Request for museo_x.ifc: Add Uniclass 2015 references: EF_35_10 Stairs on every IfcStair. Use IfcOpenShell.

First a look at what the model holds.

```python
import ifcopenshell

model = ifcopenshell.open("museo_x.ifc")
print(model.schema)
print("classifications:", [c.Name for c in model.by_type("IfcClassification")])
for ifc_class in ("IfcDoor", "IfcRoof", "IfcStair", "IfcWall", "IfcWindow"):
    print(ifc_class, len(model.by_type(ifc_class)))
```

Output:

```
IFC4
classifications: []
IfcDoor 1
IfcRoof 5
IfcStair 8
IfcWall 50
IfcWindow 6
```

```python
import ifcopenshell
import ifcopenshell.api.classification

model = ifcopenshell.open("museo_x.ifc")

system = ifcopenshell.api.classification.add_classification(model, classification="Uniclass 2015")

codes = {
    "IfcStair": ("EF_35_10", "Stairs"),
}
for ifc_class, (code, name) in codes.items():
    products = model.by_type(ifc_class)
    ifcopenshell.api.classification.add_reference(
        model, products=products, classification=system, identification=code, name=name
    )
    print(code, len(products))

model.write("museo_x-out.ifc")
```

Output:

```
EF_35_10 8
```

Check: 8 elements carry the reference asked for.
